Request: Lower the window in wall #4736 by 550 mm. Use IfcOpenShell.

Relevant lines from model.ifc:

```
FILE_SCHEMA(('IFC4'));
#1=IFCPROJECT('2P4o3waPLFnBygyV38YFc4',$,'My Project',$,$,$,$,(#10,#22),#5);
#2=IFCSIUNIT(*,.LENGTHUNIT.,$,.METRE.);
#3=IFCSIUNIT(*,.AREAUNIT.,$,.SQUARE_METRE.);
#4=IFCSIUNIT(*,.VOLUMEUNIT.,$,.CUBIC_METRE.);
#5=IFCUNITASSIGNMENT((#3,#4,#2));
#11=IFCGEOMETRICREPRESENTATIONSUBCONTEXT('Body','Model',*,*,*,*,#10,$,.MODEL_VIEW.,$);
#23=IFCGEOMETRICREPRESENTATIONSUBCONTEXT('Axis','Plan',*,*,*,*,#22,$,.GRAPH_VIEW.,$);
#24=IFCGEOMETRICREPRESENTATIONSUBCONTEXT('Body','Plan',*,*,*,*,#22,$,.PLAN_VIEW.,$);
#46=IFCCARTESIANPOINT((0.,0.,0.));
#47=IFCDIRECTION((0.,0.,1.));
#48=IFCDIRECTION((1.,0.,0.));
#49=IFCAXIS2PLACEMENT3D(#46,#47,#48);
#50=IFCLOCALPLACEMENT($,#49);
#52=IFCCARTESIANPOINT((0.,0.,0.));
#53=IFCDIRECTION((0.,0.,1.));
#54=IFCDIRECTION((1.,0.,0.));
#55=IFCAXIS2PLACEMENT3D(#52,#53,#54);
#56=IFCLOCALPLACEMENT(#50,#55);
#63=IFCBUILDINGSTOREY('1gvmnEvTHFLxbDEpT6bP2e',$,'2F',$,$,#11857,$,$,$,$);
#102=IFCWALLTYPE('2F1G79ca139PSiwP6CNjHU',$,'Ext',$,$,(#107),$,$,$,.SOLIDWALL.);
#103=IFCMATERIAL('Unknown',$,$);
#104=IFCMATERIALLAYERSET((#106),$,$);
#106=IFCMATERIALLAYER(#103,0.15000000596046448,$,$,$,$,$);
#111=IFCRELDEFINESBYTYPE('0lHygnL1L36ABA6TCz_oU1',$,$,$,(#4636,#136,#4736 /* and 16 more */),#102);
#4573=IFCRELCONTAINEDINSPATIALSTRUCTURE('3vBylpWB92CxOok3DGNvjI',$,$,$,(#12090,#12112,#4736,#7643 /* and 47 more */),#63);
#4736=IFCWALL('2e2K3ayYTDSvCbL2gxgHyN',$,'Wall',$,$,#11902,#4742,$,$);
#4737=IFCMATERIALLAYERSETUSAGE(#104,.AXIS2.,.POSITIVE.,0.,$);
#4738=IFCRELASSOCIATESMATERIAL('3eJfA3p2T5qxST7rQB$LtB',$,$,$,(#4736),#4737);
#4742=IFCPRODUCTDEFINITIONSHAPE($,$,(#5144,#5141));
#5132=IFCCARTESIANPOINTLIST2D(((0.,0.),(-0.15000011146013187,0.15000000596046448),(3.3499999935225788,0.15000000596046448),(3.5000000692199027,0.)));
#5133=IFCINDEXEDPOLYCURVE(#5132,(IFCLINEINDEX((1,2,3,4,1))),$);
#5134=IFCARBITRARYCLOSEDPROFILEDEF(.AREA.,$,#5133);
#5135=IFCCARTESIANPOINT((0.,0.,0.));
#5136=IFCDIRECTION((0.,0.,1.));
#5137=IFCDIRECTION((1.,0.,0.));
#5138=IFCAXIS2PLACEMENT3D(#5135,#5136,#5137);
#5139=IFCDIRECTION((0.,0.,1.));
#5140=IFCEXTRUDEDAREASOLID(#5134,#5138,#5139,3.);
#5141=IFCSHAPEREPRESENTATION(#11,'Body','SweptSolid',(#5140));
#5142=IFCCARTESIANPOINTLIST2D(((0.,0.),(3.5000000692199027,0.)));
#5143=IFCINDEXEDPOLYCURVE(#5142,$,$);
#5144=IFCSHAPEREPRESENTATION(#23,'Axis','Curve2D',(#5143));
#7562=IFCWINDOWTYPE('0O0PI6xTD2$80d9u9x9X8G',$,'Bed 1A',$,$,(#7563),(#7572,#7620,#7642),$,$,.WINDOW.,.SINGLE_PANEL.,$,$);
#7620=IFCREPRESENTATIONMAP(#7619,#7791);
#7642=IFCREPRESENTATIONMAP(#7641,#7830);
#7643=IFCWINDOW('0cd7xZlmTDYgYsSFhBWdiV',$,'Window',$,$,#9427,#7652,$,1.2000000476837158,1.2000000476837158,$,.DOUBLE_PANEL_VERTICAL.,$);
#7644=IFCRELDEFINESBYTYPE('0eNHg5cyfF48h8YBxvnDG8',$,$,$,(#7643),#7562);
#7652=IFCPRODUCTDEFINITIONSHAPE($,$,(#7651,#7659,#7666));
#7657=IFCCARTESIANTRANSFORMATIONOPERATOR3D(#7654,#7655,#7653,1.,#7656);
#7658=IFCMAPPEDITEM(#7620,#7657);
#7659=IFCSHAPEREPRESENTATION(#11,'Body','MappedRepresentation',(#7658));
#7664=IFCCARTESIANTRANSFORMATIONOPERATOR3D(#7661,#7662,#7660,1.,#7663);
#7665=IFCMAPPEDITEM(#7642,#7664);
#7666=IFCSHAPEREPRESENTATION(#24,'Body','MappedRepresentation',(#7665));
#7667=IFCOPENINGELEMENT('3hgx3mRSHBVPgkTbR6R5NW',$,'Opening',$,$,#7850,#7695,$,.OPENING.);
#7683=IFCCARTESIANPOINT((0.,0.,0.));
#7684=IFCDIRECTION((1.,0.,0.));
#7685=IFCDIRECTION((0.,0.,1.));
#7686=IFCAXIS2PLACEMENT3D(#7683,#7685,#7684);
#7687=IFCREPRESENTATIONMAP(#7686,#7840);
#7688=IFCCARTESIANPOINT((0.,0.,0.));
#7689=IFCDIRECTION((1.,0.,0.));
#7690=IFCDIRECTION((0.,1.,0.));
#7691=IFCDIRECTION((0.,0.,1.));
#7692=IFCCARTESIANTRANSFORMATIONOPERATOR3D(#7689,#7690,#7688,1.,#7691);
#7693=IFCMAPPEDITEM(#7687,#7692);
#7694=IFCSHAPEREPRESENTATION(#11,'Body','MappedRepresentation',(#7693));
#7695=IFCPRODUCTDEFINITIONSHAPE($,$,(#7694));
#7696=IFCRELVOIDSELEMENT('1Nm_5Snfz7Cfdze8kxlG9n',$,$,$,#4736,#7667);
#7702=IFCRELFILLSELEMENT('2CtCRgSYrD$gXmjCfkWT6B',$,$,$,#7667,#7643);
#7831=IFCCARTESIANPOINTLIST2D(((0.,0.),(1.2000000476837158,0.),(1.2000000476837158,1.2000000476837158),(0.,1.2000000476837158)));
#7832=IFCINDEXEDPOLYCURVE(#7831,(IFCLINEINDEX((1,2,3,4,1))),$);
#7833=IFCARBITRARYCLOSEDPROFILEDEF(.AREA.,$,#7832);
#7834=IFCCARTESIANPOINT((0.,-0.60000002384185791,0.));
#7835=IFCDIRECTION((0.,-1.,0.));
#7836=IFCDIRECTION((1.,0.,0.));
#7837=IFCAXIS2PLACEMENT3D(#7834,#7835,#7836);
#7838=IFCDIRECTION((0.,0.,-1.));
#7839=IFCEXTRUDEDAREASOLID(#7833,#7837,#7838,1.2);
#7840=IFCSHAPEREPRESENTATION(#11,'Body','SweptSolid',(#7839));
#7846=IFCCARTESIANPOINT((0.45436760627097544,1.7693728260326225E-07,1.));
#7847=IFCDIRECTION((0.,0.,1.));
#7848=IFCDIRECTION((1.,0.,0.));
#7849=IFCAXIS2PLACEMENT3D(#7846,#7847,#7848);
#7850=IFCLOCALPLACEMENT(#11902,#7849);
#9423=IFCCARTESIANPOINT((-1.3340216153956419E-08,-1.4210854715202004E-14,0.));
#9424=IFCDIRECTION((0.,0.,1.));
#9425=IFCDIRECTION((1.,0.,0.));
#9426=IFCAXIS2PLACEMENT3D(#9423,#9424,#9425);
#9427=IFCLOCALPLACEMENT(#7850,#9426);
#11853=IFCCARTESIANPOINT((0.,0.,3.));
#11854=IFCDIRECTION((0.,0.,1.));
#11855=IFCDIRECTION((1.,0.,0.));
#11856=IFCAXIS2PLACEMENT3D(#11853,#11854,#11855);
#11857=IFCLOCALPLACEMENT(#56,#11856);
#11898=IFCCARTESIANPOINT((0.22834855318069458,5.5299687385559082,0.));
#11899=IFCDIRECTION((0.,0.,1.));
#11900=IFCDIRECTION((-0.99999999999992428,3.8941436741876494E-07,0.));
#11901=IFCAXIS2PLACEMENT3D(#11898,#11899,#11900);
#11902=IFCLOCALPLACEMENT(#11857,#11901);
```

```python
import numpy as np
import ifcopenshell
import ifcopenshell.api.geometry
import ifcopenshell.util.placement
import ifcopenshell.util.unit

model = ifcopenshell.open("model.ifc")
unit_scale = ifcopenshell.util.unit.calculate_unit_scale(model)

window = model.by_id(7643)
opening = window.FillsVoids[0].RelatingOpeningElement
dz = -0.55 / unit_scale

shift = np.array([0.0, 0.0, dz])
# The window is placed relative to its opening, so it follows when the opening moves.
matrix = ifcopenshell.util.placement.get_local_placement(opening.ObjectPlacement)
matrix[:3, 3] += shift
ifcopenshell.api.geometry.edit_object_placement(
    model, product=opening, matrix=matrix, is_si=False, should_transform_children=True
)

print(f"moved by {dz * unit_scale:+.3f} m")

model.write("model_v2.ifc")
```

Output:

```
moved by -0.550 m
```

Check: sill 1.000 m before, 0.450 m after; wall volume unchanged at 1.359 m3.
